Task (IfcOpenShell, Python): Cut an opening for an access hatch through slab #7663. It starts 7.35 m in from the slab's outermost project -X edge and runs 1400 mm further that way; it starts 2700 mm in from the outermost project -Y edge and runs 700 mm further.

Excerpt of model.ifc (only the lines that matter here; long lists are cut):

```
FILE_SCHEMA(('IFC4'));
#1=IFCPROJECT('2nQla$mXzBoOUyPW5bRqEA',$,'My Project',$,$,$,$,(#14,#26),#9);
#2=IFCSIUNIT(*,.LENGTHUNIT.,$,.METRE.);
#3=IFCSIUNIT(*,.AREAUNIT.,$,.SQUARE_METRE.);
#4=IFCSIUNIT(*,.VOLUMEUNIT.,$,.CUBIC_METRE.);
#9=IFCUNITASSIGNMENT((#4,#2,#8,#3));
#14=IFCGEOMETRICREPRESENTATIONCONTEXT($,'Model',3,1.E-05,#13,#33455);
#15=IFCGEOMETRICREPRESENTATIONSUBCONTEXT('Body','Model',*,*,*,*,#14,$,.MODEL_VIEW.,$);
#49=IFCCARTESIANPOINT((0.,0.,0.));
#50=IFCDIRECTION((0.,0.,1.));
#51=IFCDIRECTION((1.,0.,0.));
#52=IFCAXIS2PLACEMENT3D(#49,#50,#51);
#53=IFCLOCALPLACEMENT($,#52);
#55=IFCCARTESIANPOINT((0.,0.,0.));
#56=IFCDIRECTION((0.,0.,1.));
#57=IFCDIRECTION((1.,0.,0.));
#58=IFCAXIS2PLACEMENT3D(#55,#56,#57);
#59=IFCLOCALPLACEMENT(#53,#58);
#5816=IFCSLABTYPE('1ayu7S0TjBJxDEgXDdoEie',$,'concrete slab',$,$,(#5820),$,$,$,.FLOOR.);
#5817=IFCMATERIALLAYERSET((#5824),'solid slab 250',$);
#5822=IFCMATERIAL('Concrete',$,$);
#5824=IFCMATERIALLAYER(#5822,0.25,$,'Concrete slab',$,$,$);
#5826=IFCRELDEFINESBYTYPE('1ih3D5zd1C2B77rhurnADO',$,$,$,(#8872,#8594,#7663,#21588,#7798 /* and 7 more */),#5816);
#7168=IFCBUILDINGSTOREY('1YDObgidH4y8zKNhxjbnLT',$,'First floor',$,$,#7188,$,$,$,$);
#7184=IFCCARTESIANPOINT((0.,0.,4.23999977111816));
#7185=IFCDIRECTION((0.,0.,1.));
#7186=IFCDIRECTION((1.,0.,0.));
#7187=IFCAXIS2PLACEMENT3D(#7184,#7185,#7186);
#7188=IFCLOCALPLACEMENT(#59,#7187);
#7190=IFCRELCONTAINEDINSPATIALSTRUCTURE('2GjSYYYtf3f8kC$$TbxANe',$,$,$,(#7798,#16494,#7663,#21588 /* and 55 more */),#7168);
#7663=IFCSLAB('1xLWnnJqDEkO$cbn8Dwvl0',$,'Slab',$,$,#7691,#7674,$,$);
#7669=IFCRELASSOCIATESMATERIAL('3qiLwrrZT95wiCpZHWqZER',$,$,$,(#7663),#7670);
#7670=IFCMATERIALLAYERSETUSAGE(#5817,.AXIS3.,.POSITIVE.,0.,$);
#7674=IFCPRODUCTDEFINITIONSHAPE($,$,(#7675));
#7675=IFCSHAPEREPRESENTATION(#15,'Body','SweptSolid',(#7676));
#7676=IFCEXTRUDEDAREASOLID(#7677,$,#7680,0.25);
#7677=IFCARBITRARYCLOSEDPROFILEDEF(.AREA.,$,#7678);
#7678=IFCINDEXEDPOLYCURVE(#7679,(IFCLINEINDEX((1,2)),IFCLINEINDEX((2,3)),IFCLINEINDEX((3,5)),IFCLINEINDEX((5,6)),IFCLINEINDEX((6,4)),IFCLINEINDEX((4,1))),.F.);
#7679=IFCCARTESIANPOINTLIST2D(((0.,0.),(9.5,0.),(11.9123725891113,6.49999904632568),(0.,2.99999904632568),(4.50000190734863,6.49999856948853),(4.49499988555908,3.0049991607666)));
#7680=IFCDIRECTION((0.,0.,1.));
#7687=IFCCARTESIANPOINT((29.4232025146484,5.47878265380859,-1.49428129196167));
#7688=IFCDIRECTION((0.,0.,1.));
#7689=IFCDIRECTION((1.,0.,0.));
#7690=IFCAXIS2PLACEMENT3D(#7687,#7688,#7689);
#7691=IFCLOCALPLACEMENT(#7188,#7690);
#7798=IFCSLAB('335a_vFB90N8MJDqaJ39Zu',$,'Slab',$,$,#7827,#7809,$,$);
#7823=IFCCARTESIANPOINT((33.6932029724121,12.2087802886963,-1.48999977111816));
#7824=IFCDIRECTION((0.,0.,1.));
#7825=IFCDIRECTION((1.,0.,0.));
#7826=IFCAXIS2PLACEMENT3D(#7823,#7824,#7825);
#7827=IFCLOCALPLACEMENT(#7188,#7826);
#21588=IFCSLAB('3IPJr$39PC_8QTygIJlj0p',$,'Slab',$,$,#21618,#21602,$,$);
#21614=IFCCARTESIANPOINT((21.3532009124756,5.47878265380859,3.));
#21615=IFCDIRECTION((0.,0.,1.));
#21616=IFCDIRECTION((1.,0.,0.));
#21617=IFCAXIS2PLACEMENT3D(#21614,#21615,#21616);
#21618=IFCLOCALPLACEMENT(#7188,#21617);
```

```python
import numpy as np
import ifcopenshell
import ifcopenshell.api.feature
import ifcopenshell.api.geometry
import ifcopenshell.api.root
import ifcopenshell.geom
import ifcopenshell.util.placement
import ifcopenshell.util.representation
import ifcopenshell.util.shape
import ifcopenshell.util.unit

model = ifcopenshell.open("model.ifc")
unit_scale = ifcopenshell.util.unit.calculate_unit_scale(model)
settings = ifcopenshell.geom.settings()


def volume(element):
    """Net volume in cubic metres, openings subtracted."""
    shape = ifcopenshell.geom.create_shape(settings, element)
    return ifcopenshell.util.shape.get_volume(shape.geometry)


slab = model.by_guid("1xLWnnJqDEkO$cbn8Dwvl0")
before = volume(slab)

# Extent in the slab's own axes, in metres. The edges named are its -X and -Y sides.
slab_shape = ifcopenshell.geom.create_shape(settings, slab)
vertices = ifcopenshell.util.shape.get_vertices(slab_shape.geometry)
x_min, y_min, bottom = vertices.min(axis=0)
top = vertices[:, 2].max()

opening = ifcopenshell.api.root.create_entity(model, ifc_class="IfcOpeningElement", name="Access hatch opening", predefined_type="OPENING")
context = ifcopenshell.util.representation.get_context(model, "Model", "Body", "MODEL_VIEW")
width, depth = 1.4, 0.7
outline = [(0.0, 0.0), (width, 0.0), (width, depth), (0.0, depth), (0.0, 0.0)]
# Overshoot both faces by 50 mm so the cut is clean.
shape = ifcopenshell.api.geometry.add_slab_representation(
    model, context=context, depth=top - bottom + 0.1, polyline=outline
)
ifcopenshell.api.geometry.assign_representation(model, product=opening, representation=shape)

matrix = ifcopenshell.util.placement.get_local_placement(slab.ObjectPlacement)
matrix[:, 3] = matrix @ np.append(np.array([x_min + 7.35, y_min + 2.7, bottom - 0.05]) / unit_scale, 1.0)
ifcopenshell.api.geometry.edit_object_placement(model, product=opening, matrix=matrix, is_si=False)
ifcopenshell.api.feature.add_feature(model, feature=opening, element=slab)

after = volume(slab)

print(f"slab volume {before:.3f} -> {after:.3f} m3")

model.write("model-out.ifc")
```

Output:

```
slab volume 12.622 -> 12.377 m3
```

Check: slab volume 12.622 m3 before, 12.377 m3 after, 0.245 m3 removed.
